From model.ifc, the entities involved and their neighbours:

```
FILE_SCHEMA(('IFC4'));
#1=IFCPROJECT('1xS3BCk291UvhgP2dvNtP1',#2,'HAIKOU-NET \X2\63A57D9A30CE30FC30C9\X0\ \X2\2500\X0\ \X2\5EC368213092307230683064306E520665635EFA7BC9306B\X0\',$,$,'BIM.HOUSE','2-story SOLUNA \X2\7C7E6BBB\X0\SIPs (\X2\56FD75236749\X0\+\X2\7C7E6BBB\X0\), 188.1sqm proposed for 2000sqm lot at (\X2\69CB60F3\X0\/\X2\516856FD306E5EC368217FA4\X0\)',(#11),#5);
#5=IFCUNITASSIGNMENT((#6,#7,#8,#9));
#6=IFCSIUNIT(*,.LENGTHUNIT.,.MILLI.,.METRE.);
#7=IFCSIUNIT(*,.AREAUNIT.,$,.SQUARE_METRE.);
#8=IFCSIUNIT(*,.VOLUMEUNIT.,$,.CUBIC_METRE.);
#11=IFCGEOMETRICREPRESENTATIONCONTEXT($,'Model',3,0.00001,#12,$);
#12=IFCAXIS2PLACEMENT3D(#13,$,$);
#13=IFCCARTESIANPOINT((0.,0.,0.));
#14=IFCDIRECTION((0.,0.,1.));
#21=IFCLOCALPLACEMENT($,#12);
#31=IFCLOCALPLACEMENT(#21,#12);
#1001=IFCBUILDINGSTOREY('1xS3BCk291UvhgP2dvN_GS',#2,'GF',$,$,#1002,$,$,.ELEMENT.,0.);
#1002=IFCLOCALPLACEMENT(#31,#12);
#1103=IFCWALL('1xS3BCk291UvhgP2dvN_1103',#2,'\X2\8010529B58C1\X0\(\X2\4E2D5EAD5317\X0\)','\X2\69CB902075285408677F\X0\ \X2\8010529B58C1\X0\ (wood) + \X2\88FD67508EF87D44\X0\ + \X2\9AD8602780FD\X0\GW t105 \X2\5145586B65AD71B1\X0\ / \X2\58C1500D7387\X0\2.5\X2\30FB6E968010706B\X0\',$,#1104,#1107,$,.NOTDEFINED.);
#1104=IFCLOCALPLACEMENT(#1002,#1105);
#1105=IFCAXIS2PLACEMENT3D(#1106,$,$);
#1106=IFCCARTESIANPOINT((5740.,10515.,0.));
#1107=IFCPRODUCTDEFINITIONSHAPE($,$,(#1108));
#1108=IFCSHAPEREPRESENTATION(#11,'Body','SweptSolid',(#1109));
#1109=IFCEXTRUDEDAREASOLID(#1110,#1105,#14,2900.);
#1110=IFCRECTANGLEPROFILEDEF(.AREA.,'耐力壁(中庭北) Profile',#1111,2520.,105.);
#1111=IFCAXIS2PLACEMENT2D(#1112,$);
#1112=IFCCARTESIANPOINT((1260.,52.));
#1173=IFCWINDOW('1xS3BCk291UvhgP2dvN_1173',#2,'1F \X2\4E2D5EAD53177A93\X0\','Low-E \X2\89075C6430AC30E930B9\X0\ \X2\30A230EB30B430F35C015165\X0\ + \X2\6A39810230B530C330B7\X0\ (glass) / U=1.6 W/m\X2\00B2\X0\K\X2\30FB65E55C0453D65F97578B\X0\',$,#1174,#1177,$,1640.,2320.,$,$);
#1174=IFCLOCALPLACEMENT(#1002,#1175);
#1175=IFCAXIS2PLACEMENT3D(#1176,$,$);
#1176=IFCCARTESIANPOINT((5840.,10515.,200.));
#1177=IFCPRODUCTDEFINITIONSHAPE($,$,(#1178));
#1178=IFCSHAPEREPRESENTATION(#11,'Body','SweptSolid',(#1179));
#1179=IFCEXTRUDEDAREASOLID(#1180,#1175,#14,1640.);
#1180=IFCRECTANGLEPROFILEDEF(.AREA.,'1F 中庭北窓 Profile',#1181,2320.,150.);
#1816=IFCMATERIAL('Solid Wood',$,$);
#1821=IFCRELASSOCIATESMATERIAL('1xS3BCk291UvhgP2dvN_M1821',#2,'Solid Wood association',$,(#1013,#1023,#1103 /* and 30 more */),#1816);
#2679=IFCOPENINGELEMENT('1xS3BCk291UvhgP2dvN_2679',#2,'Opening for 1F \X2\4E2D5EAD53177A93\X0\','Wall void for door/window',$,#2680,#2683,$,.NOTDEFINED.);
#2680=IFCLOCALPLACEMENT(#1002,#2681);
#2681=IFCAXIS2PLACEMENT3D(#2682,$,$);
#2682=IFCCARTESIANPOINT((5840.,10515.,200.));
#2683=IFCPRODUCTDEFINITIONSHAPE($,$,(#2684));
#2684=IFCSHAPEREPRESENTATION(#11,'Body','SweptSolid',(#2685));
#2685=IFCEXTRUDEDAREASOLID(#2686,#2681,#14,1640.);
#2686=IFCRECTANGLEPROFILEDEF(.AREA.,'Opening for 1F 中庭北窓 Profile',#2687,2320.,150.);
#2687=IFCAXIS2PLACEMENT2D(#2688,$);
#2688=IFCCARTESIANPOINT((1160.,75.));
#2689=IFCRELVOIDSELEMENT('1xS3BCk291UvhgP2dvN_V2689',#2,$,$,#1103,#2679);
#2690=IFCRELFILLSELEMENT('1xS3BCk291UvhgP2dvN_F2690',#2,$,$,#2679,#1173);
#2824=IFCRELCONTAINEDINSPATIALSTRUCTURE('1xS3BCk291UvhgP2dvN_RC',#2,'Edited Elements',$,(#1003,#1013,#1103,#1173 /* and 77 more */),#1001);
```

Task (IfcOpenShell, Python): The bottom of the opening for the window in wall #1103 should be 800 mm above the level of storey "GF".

```python
import numpy as np
import ifcopenshell
import ifcopenshell.api.geometry
import ifcopenshell.geom
import ifcopenshell.util.element
import ifcopenshell.util.placement
import ifcopenshell.util.shape
import ifcopenshell.util.unit

model = ifcopenshell.open("model.ifc")
unit_scale = ifcopenshell.util.unit.calculate_unit_scale(model)

window = model.by_guid("1xS3BCk291UvhgP2dvN_1173")
opening = window.FillsVoids[0].RelatingOpeningElement
storey = ifcopenshell.util.element.get_container(window, ifc_class="IfcBuildingStorey")
level = ifcopenshell.util.placement.get_local_placement(storey.ObjectPlacement)[2, 3]

# The opening's origin need not be at the sill, so measure its lowest point.
shape = ifcopenshell.geom.create_shape(ifcopenshell.geom.settings(), opening)
bottom = ifcopenshell.util.shape.get_shape_bottom_elevation(shape, shape.geometry) / unit_scale
dz = level + 800.0 - bottom

shift = np.array([0.0, 0.0, dz])
# The window is not placed relative to its opening, so move both.
for product in (opening, window):
    matrix = ifcopenshell.util.placement.get_local_placement(product.ObjectPlacement)
    matrix[:3, 3] += shift
    ifcopenshell.api.geometry.edit_object_placement(model, product=product, matrix=matrix, is_si=False)

print(f"moved by {dz * unit_scale:+.3f} m")

model.write("model_edited.ifc")
```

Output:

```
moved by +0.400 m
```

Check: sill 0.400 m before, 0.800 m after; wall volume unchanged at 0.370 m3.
